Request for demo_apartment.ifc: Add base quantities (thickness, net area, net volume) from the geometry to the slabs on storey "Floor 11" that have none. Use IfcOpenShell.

First a look at what the model holds.

```python
import ifcopenshell
import ifcopenshell.util.element
import ifcopenshell.util.unit

model = ifcopenshell.open("demo_apartment.ifc")
print(model.schema)
for unit_type in ("LENGTHUNIT", "AREAUNIT", "VOLUMEUNIT"):
    print(unit_type, ifcopenshell.util.unit.calculate_unit_scale(model, unit_type))
storey = next(s for s in model.by_type("IfcBuildingStorey") if s.Name == "Floor 11")
slabs = [e for e in ifcopenshell.util.element.get_decomposition(storey) if e.is_a("IfcSlab")]
for e in sorted(slabs, key=lambda e: e.id()):
    print(e.id(), e.is_a(), e.Name, list(ifcopenshell.util.element.get_psets(e, qtos_only=True)), sep=" | ")
```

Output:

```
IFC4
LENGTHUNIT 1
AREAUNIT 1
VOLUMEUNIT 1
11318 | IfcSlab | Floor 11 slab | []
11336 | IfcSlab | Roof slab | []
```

```python
import ifcopenshell
import ifcopenshell.api.pset
import ifcopenshell.geom
import ifcopenshell.util.element
import ifcopenshell.util.shape
import ifcopenshell.util.unit

model = ifcopenshell.open("demo_apartment.ifc")
unit_scale = ifcopenshell.util.unit.calculate_unit_scale(model)
area_scale = ifcopenshell.util.unit.calculate_unit_scale(model, "AREAUNIT")
volume_scale = ifcopenshell.util.unit.calculate_unit_scale(model, "VOLUMEUNIT")
settings = ifcopenshell.geom.settings()

storey = next(s for s in model.by_type("IfcBuildingStorey") if s.Name == "Floor 11")
slabs = [e for e in ifcopenshell.util.element.get_decomposition(storey) if e.is_a("IfcSlab")]

for e in sorted(slabs, key=lambda e: e.id()):
    if ifcopenshell.util.element.get_psets(e, qtos_only=True, should_inherit=False):
        continue
    # Geometry comes back in metres, in the element's own axes.
    shape = ifcopenshell.geom.create_shape(settings, e)
    values = {
        "Width": ifcopenshell.util.shape.get_z(shape.geometry) / unit_scale,
        "NetArea": ifcopenshell.util.shape.get_footprint_area(shape.geometry) / area_scale,
        "NetVolume": ifcopenshell.util.shape.get_volume(shape.geometry) / volume_scale,
    }
    qto = ifcopenshell.api.pset.add_qto(model, product=e, name="Qto_SlabBaseQuantities")
    ifcopenshell.api.pset.edit_qto(model, qto=qto, properties=values)
    print(e.id(), {k: round(v, 3) for k, v in values.items()})

model.write("demo_apartment_rev.ifc")
```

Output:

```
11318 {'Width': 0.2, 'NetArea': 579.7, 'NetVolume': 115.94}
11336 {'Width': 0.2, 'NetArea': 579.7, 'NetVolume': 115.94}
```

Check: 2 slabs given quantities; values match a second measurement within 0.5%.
